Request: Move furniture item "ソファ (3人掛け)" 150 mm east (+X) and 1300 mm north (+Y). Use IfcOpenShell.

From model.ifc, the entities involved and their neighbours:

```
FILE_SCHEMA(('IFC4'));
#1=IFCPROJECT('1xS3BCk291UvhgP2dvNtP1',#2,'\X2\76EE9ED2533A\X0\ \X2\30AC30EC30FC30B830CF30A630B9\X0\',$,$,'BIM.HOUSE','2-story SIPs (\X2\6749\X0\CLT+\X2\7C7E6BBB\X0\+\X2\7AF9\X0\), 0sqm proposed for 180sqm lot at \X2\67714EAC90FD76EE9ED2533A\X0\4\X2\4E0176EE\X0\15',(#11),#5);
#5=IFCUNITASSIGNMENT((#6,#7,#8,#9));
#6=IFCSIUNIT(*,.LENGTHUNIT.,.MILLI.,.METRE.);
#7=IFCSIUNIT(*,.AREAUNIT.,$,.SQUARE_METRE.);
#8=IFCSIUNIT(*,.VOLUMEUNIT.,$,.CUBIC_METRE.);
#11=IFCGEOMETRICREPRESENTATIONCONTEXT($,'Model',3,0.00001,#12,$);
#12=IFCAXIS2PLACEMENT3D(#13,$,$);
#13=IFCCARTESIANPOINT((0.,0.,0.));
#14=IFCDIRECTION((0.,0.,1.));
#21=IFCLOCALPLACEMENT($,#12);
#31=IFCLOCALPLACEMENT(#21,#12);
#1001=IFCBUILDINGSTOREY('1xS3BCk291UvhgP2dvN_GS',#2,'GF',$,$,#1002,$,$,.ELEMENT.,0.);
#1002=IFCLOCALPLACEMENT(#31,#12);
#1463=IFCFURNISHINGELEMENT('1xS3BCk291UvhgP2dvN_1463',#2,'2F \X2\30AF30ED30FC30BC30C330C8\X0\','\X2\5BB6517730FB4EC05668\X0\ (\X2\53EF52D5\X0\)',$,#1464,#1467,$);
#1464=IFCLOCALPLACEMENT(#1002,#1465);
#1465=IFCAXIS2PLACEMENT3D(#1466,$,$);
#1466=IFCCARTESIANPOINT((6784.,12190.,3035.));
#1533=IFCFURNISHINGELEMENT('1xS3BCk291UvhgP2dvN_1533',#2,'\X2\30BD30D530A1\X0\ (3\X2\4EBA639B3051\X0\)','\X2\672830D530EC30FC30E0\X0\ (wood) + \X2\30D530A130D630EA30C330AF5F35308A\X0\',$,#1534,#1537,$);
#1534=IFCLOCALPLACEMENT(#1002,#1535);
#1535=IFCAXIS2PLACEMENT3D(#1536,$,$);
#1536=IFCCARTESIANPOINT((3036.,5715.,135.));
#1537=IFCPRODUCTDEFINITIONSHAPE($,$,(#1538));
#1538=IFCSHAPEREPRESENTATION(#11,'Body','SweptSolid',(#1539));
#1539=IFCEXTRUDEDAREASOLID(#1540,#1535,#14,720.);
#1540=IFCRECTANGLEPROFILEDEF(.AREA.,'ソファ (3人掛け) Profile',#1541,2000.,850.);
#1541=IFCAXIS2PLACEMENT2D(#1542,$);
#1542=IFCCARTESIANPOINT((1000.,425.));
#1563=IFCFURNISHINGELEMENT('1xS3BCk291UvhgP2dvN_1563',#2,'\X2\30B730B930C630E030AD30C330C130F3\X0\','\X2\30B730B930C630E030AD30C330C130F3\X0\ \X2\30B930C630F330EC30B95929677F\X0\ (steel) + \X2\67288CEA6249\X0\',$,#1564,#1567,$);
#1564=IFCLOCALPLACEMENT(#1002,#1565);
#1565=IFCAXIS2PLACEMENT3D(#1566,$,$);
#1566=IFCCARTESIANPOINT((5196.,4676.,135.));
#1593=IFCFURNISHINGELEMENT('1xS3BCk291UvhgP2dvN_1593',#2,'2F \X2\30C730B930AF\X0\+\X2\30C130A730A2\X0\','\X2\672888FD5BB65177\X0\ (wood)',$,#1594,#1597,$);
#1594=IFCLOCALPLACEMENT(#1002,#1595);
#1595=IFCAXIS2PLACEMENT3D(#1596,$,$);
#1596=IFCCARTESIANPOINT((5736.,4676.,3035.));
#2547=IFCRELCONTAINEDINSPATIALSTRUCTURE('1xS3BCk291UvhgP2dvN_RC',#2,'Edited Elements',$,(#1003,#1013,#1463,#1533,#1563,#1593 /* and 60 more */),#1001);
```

```python
import ifcopenshell
import ifcopenshell.api.geometry
import ifcopenshell.util.placement
import ifcopenshell.util.unit

model = ifcopenshell.open("model.ifc")
unit_scale = ifcopenshell.util.unit.calculate_unit_scale(model)

item = model.by_guid("1xS3BCk291UvhgP2dvN_1533")
matrix = ifcopenshell.util.placement.get_local_placement(item.ObjectPlacement)
matrix[0, 3] += 0.15 / unit_scale
matrix[1, 3] += 1.3 / unit_scale
ifcopenshell.api.geometry.edit_object_placement(model, product=item, matrix=matrix, is_si=False)

print(ifcopenshell.util.placement.get_local_placement(item.ObjectPlacement).round(3) + 0.0)

model.write("model_edited.ifc")
```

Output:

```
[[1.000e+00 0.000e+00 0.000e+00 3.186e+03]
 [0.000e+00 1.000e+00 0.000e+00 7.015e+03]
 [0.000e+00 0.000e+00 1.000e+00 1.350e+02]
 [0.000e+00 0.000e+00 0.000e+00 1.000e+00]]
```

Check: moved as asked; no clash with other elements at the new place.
